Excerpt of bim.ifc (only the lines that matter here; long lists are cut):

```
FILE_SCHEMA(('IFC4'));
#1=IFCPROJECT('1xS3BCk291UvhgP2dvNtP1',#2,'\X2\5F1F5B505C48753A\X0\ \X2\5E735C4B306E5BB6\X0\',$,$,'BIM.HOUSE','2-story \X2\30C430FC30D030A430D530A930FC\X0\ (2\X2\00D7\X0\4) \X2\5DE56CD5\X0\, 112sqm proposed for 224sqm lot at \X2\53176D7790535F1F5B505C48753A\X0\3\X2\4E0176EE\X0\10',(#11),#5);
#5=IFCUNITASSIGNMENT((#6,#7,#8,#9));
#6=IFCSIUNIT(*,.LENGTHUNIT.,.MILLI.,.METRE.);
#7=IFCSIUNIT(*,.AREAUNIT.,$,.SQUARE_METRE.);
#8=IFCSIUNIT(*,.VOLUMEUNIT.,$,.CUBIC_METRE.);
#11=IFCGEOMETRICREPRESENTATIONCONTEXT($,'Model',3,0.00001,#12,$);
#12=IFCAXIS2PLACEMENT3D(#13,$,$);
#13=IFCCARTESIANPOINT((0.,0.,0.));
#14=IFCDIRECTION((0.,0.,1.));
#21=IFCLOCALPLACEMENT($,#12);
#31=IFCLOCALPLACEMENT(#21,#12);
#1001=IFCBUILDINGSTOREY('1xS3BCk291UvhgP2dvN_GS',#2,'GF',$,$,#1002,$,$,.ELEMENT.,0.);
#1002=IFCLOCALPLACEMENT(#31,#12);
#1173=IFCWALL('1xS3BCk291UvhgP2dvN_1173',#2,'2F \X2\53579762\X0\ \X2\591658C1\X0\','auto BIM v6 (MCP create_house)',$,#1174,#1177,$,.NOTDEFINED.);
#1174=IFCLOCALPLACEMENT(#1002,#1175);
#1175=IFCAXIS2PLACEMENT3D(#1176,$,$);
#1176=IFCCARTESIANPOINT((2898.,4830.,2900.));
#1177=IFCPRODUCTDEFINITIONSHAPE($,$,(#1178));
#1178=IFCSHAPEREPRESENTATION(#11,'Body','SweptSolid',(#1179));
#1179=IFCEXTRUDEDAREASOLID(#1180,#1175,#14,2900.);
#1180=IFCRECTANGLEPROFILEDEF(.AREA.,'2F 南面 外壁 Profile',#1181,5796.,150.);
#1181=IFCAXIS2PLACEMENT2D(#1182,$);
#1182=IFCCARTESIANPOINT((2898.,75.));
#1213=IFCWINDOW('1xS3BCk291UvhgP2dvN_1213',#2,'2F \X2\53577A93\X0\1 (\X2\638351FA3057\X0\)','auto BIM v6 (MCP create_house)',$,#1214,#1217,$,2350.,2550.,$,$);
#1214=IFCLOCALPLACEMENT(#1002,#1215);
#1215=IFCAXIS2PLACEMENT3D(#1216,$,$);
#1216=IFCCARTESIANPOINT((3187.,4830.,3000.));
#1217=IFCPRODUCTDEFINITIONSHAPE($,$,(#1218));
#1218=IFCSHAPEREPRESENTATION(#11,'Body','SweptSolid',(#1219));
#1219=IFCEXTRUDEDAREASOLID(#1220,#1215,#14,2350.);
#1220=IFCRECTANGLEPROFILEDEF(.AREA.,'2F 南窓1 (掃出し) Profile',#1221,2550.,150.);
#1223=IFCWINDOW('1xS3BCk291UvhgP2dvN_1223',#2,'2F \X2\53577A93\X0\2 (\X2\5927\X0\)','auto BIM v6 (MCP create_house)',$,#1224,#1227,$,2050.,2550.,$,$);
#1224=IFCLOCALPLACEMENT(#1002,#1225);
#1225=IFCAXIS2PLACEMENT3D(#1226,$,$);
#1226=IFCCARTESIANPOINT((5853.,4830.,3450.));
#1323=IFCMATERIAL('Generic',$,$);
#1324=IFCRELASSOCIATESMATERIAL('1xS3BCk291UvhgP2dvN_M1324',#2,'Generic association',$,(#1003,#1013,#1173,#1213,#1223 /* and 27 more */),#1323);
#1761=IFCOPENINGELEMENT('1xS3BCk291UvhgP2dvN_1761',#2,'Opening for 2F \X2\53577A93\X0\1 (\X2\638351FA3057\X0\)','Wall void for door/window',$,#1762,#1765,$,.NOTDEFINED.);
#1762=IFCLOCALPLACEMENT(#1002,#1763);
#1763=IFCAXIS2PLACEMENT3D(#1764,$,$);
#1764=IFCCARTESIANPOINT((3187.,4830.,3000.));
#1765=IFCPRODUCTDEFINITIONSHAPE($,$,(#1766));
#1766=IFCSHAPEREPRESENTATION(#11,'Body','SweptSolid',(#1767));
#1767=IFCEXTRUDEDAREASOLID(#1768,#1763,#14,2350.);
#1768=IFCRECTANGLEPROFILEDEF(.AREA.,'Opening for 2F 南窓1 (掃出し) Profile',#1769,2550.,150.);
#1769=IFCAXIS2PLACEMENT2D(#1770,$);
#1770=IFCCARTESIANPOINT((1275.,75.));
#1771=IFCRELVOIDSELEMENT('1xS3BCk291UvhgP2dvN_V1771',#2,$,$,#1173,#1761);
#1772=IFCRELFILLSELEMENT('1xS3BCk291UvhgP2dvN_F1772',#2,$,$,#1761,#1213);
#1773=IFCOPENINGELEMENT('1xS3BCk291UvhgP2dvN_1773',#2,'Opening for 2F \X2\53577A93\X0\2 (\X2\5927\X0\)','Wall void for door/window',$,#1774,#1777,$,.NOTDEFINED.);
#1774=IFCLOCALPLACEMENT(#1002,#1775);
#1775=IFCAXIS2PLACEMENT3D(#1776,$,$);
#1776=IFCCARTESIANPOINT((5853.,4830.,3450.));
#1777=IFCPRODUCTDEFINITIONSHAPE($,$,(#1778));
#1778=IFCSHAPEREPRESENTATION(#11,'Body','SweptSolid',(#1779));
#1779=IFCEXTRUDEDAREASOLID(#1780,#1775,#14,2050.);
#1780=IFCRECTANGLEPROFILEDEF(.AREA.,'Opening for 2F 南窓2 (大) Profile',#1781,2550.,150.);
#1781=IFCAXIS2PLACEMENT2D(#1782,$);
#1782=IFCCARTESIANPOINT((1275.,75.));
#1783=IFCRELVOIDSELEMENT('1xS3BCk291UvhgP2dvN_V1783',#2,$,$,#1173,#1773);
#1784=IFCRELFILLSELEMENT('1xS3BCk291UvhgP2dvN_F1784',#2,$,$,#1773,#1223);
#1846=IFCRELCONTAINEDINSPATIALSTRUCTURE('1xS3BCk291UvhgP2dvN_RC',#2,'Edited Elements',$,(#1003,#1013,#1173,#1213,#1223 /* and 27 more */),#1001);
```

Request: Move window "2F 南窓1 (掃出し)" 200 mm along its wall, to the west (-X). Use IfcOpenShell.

```python
import ifcopenshell
import ifcopenshell.api.geometry
import ifcopenshell.util.placement

model = ifcopenshell.open("bim.ifc")

window = model.by_guid("1xS3BCk291UvhgP2dvN_1213")
opening = window.FillsVoids[0].RelatingOpeningElement
wall = opening.VoidsElements[0].RelatingBuildingElement

wall_matrix = ifcopenshell.util.placement.get_local_placement(wall.ObjectPlacement)
shift = wall_matrix[:3, 0] * -200.0
before = ifcopenshell.util.placement.get_local_placement(window.ObjectPlacement)[:3, 3].copy()

# The window is not placed relative to its opening, so move both.
for product in (opening, window):
    matrix = ifcopenshell.util.placement.get_local_placement(product.ObjectPlacement)
    matrix[:3, 3] += shift
    ifcopenshell.api.geometry.edit_object_placement(model, product=product, matrix=matrix, is_si=False)

after = ifcopenshell.util.placement.get_local_placement(window.ObjectPlacement)[:3, 3]
print("window moved by", (after - before).round(3) + 0.0)

model.write("bim_v2.ifc")
```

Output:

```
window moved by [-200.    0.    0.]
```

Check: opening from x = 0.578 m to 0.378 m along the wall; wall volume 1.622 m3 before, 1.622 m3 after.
